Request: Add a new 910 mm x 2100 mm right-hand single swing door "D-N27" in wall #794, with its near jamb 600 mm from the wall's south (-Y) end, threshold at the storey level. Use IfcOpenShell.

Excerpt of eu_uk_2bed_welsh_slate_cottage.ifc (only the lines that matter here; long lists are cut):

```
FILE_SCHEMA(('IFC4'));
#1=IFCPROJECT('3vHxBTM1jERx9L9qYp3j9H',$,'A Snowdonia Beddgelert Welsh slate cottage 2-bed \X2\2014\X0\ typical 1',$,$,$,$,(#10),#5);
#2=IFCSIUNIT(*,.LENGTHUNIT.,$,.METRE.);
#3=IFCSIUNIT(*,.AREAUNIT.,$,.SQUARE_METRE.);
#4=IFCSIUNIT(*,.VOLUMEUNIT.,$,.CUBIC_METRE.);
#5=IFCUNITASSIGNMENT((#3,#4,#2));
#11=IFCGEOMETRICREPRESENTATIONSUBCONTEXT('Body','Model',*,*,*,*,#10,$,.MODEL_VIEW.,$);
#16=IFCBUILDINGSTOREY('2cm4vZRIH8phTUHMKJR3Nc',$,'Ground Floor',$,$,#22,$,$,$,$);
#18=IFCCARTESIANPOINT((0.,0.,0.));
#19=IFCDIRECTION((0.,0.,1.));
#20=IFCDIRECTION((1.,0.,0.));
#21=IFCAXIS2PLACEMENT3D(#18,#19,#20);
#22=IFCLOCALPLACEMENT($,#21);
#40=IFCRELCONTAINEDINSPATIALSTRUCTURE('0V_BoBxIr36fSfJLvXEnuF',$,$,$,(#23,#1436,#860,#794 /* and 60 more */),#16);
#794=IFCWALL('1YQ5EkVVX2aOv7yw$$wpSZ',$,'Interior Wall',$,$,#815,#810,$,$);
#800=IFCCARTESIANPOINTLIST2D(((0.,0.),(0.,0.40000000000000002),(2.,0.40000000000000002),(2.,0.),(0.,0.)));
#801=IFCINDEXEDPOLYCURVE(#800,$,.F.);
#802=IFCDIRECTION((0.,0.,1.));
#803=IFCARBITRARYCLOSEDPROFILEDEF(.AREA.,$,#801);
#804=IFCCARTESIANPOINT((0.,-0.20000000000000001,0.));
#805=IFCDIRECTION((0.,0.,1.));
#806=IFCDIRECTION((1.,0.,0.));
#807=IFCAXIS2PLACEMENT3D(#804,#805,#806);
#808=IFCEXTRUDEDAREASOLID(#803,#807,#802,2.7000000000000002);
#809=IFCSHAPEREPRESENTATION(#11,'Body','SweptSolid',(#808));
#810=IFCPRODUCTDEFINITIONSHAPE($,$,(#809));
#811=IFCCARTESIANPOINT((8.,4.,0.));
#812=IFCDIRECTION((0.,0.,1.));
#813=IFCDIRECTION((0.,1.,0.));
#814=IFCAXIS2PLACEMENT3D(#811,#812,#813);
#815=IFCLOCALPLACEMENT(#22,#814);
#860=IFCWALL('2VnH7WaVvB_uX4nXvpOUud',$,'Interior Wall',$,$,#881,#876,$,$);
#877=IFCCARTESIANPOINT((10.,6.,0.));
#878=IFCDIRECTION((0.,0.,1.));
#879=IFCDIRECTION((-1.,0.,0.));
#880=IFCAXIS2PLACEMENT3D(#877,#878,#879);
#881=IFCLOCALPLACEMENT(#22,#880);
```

```python
import numpy as np
import ifcopenshell
import ifcopenshell.api.feature
import ifcopenshell.api.geometry
import ifcopenshell.api.root
import ifcopenshell.api.spatial
import ifcopenshell.geom
import ifcopenshell.util.element
import ifcopenshell.util.placement
import ifcopenshell.util.representation
import ifcopenshell.util.shape
import ifcopenshell.util.unit

model = ifcopenshell.open("eu_uk_2bed_welsh_slate_cottage.ifc")
unit_scale = ifcopenshell.util.unit.calculate_unit_scale(model)
settings = ifcopenshell.geom.settings()


def volume(element):
    """Net volume in cubic metres, openings subtracted."""
    shape = ifcopenshell.geom.create_shape(settings, element)
    return ifcopenshell.util.shape.get_volume(shape.geometry)


wall = model.by_guid("1YQ5EkVVX2aOv7yw$$wpSZ")
storey = ifcopenshell.util.element.get_container(wall, ifc_class="IfcBuildingStorey")
context = ifcopenshell.util.representation.get_context(model, "Model", "Body", "MODEL_VIEW")
before = volume(wall)

width, height, from_end, sill = 0.91, 2.1, 0.6, 0.0  # metres

# The wall runs along its own X axis, and the end named is its -X end.
wall_shape = ifcopenshell.geom.create_shape(settings, wall)
x, y, z = ifcopenshell.util.shape.get_vertices(wall_shape.geometry).T
start = x.min() + from_end
face, thickness = float(y.min()), float(y.max() - y.min())
wall_matrix = ifcopenshell.util.placement.get_local_placement(wall.ObjectPlacement)
level = ifcopenshell.util.placement.get_local_placement(storey.ObjectPlacement)[2, 3]


def in_wall(x, y):
    """Placement at x, y metres in the wall's axes, at sill height."""
    matrix = wall_matrix.copy()
    matrix[:, 3] = wall_matrix @ np.array([x / unit_scale, y / unit_scale, 0.0, 1.0])
    matrix[2, 3] = level + sill / unit_scale
    return matrix


# Opening: a box that overshoots both wall faces by 50 mm.
opening = ifcopenshell.api.root.create_entity(model, ifc_class="IfcOpeningElement", predefined_type="OPENING")
box = ifcopenshell.api.geometry.add_wall_representation(
    model, context=context, length=width, height=height, thickness=thickness + 0.1
)
ifcopenshell.api.geometry.assign_representation(model, product=opening, representation=box)
ifcopenshell.api.geometry.edit_object_placement(model, product=opening, matrix=in_wall(start, face - 0.05), is_si=False)
ifcopenshell.api.feature.add_feature(model, feature=opening, element=wall)

door = ifcopenshell.api.root.create_entity(model, ifc_class="IfcDoor", name="D-N27", predefined_type="DOOR")
door.OverallWidth, door.OverallHeight = width / unit_scale, height / unit_scale
door.OperationType = "SINGLE_SWING_RIGHT"
body = ifcopenshell.api.geometry.add_door_representation(
    model,
    context=context,
    overall_width=door.OverallWidth,
    overall_height=door.OverallHeight,
    operation_type="SINGLE_SWING_RIGHT",
    lining_properties={"LiningDepth": thickness / unit_scale, "ThresholdDepth": thickness / unit_scale},
)
ifcopenshell.api.geometry.assign_representation(model, product=door, representation=body)
ifcopenshell.api.spatial.assign_container(model, products=[door], relating_structure=storey)
ifcopenshell.api.feature.add_filling(model, opening=opening, element=door)

# The lining spans the wall, so the door starts at the wall face.
ifcopenshell.api.geometry.edit_object_placement(model, product=door, matrix=in_wall(start, face), is_si=False)

after = volume(wall)

print(f"wall volume {before:.3f} -> {after:.3f} m3")

model.write("eu_uk_2bed_welsh_slate_cottage_edited.ifc")
```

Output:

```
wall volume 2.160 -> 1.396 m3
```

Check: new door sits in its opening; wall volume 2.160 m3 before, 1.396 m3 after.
